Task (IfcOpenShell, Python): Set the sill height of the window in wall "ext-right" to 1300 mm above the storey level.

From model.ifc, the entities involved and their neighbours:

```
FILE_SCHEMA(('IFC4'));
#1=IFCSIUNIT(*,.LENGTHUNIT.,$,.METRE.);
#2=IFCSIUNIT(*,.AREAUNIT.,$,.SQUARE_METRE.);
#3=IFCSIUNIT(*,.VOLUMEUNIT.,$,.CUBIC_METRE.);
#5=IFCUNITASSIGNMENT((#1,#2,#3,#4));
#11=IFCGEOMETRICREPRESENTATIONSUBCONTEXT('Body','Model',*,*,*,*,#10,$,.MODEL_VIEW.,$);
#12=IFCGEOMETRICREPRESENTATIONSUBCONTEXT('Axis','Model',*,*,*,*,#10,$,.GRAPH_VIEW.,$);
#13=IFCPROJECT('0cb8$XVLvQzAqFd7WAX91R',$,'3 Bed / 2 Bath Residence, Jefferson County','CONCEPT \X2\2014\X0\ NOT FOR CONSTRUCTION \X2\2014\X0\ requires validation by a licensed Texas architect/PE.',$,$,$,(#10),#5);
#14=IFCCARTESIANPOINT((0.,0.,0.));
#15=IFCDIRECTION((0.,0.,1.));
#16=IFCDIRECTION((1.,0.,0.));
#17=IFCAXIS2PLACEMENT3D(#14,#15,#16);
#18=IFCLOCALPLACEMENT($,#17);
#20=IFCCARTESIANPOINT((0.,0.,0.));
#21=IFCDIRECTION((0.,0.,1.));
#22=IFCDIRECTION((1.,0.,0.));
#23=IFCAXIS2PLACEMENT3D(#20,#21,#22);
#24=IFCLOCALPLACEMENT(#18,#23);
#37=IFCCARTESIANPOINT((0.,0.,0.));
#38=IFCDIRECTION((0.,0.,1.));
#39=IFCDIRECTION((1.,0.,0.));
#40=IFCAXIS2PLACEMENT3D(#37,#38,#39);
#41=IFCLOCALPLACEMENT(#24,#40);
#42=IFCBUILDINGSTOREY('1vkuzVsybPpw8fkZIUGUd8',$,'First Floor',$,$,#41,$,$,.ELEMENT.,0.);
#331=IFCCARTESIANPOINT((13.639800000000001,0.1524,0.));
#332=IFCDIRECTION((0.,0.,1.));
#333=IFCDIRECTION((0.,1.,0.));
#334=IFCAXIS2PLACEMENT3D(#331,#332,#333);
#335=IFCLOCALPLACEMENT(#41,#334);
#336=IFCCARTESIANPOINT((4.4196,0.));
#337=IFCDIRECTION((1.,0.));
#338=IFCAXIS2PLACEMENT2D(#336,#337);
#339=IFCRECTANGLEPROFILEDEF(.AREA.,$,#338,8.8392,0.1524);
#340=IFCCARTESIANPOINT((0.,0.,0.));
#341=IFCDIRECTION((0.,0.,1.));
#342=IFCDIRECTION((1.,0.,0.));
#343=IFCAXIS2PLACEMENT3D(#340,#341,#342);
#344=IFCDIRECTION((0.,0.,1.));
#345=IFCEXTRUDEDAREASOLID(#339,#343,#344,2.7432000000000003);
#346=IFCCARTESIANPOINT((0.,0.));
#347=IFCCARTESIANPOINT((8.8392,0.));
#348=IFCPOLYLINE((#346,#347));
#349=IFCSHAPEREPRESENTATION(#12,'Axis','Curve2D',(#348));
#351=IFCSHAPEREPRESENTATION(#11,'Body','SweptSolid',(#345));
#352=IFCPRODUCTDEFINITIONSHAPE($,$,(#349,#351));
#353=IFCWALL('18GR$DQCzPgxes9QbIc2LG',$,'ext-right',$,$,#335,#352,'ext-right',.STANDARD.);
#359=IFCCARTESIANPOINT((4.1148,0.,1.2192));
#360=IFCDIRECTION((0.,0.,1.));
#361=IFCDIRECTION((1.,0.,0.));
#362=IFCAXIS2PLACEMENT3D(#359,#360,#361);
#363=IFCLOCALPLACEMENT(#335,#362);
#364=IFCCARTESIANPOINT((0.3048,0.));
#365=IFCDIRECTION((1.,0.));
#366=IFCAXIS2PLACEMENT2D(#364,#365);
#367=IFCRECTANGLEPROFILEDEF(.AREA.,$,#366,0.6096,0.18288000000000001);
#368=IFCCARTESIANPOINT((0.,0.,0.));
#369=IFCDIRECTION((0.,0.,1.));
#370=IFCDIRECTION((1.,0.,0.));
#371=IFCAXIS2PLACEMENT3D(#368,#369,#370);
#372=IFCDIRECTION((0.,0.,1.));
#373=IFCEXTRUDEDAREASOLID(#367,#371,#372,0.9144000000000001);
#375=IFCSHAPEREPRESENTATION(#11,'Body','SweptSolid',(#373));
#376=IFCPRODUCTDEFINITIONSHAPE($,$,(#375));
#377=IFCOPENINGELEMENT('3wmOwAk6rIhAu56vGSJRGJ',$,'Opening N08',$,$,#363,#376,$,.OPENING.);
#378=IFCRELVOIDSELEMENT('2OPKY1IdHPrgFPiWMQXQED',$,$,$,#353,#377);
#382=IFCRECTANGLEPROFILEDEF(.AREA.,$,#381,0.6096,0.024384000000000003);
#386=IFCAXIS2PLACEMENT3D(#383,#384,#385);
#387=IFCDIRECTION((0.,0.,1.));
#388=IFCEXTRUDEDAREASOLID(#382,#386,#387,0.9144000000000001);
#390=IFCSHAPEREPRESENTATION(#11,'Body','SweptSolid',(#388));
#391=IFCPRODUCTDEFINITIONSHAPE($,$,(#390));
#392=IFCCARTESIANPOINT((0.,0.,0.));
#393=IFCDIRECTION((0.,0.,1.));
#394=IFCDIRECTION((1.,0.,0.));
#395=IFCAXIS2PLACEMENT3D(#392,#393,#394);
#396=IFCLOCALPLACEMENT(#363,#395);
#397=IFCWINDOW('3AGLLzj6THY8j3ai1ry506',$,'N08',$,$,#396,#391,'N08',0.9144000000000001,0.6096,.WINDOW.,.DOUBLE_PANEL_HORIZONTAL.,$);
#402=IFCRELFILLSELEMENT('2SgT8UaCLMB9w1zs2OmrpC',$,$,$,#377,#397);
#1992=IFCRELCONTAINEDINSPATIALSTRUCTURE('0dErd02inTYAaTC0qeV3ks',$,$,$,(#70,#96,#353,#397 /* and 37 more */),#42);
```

```python
import numpy as np
import ifcopenshell
import ifcopenshell.api.geometry
import ifcopenshell.geom
import ifcopenshell.util.element
import ifcopenshell.util.placement
import ifcopenshell.util.shape
import ifcopenshell.util.unit

model = ifcopenshell.open("model.ifc")
unit_scale = ifcopenshell.util.unit.calculate_unit_scale(model)

window = model.by_guid("3AGLLzj6THY8j3ai1ry506")
opening = window.FillsVoids[0].RelatingOpeningElement
storey = ifcopenshell.util.element.get_container(window, ifc_class="IfcBuildingStorey")
level = ifcopenshell.util.placement.get_local_placement(storey.ObjectPlacement)[2, 3]

# The opening's origin need not be at the sill, so measure its lowest point.
shape = ifcopenshell.geom.create_shape(ifcopenshell.geom.settings(), opening)
bottom = ifcopenshell.util.shape.get_shape_bottom_elevation(shape, shape.geometry) / unit_scale
dz = level + 1.3 - bottom

shift = np.array([0.0, 0.0, dz])
# The window is placed relative to its opening, so it follows when the opening moves.
matrix = ifcopenshell.util.placement.get_local_placement(opening.ObjectPlacement)
matrix[:3, 3] += shift
ifcopenshell.api.geometry.edit_object_placement(
    model, product=opening, matrix=matrix, is_si=False, should_transform_children=True
)

print(f"moved by {dz * unit_scale:+.3f} m")

model.write("model_rev.ifc")
```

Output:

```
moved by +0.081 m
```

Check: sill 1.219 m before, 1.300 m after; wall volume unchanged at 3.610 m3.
